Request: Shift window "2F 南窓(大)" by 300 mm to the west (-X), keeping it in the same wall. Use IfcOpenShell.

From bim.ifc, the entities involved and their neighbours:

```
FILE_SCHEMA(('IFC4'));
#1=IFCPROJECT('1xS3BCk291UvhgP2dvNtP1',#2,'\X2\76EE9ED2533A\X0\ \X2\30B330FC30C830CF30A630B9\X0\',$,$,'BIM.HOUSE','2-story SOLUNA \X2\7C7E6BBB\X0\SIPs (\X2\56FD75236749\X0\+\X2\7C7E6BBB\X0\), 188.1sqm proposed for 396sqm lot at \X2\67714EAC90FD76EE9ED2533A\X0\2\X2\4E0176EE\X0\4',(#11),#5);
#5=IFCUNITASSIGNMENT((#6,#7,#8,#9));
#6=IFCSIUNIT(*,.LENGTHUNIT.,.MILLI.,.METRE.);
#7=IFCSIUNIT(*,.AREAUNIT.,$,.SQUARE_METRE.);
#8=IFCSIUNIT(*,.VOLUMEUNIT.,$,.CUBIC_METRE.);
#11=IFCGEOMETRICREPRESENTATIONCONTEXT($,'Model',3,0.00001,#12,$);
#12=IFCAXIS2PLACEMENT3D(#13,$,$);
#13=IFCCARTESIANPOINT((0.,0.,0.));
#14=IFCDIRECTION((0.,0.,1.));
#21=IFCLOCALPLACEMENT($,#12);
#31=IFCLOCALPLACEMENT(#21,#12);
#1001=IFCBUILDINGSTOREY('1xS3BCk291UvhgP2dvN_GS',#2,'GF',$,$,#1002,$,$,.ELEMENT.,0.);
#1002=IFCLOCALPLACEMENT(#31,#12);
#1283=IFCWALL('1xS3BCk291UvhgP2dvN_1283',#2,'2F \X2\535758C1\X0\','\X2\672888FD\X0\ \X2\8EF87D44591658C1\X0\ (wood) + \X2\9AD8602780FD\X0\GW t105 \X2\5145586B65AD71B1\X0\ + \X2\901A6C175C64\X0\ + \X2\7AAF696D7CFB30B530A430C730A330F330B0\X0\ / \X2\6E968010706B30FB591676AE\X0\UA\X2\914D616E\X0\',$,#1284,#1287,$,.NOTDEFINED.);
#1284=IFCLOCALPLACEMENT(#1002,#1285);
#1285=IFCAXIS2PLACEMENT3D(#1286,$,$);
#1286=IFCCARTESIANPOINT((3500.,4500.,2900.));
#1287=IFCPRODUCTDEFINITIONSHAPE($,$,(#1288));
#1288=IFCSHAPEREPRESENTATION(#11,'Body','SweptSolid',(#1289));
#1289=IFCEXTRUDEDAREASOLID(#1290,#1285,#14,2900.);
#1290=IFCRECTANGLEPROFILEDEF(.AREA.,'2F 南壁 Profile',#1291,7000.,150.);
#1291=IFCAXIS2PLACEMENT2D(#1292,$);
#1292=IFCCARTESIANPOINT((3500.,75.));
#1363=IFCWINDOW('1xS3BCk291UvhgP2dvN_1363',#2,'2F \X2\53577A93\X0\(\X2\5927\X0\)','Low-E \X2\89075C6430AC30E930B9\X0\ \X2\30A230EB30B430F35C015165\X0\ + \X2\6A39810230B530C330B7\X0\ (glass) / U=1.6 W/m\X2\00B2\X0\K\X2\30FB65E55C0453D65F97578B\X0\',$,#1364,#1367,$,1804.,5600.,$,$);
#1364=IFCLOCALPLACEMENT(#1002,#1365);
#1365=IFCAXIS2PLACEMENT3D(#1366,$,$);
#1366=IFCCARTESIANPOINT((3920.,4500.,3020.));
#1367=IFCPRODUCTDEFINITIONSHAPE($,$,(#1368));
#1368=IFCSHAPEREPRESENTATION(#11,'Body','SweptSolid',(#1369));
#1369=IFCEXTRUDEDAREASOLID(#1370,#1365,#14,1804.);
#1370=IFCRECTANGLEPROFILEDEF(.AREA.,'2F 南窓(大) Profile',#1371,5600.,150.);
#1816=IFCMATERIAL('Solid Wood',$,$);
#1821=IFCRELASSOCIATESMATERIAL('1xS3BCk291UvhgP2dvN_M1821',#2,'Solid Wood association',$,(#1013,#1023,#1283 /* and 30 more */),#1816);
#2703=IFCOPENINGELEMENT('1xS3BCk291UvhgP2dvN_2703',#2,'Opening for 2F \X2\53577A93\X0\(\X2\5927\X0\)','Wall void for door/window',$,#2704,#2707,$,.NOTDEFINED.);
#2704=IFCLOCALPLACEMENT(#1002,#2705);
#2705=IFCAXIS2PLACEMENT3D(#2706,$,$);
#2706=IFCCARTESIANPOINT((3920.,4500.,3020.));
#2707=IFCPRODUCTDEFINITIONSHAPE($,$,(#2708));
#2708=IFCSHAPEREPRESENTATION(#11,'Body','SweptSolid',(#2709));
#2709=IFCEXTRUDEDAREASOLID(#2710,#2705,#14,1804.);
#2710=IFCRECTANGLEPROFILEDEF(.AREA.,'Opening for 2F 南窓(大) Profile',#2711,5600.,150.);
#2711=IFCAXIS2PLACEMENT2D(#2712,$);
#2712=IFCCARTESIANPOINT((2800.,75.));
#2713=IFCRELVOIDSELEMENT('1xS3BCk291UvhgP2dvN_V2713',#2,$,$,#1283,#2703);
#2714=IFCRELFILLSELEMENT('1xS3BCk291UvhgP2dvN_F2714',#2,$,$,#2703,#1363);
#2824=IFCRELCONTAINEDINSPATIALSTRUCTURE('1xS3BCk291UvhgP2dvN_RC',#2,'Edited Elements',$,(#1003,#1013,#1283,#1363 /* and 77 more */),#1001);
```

```python
import ifcopenshell
import ifcopenshell.api.geometry
import ifcopenshell.util.placement
import ifcopenshell.util.unit

model = ifcopenshell.open("bim.ifc")
unit_scale = ifcopenshell.util.unit.calculate_unit_scale(model)

window = model.by_guid("1xS3BCk291UvhgP2dvN_1363")
opening = window.FillsVoids[0].RelatingOpeningElement
wall = opening.VoidsElements[0].RelatingBuildingElement

wall_matrix = ifcopenshell.util.placement.get_local_placement(wall.ObjectPlacement)
shift = wall_matrix[:3, 0] * -0.3 / unit_scale
before = ifcopenshell.util.placement.get_local_placement(window.ObjectPlacement)[:3, 3].copy()

# The window is not placed relative to its opening, so move both.
for product in (opening, window):
    matrix = ifcopenshell.util.placement.get_local_placement(product.ObjectPlacement)
    matrix[:3, 3] += shift
    ifcopenshell.api.geometry.edit_object_placement(model, product=product, matrix=matrix, is_si=False)

after = ifcopenshell.util.placement.get_local_placement(window.ObjectPlacement)[:3, 3]
print("window moved by", (after - before).round(3) + 0.0)

model.write("bim_edited.ifc")
```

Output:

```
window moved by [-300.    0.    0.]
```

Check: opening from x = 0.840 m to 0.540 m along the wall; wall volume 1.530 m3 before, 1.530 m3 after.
